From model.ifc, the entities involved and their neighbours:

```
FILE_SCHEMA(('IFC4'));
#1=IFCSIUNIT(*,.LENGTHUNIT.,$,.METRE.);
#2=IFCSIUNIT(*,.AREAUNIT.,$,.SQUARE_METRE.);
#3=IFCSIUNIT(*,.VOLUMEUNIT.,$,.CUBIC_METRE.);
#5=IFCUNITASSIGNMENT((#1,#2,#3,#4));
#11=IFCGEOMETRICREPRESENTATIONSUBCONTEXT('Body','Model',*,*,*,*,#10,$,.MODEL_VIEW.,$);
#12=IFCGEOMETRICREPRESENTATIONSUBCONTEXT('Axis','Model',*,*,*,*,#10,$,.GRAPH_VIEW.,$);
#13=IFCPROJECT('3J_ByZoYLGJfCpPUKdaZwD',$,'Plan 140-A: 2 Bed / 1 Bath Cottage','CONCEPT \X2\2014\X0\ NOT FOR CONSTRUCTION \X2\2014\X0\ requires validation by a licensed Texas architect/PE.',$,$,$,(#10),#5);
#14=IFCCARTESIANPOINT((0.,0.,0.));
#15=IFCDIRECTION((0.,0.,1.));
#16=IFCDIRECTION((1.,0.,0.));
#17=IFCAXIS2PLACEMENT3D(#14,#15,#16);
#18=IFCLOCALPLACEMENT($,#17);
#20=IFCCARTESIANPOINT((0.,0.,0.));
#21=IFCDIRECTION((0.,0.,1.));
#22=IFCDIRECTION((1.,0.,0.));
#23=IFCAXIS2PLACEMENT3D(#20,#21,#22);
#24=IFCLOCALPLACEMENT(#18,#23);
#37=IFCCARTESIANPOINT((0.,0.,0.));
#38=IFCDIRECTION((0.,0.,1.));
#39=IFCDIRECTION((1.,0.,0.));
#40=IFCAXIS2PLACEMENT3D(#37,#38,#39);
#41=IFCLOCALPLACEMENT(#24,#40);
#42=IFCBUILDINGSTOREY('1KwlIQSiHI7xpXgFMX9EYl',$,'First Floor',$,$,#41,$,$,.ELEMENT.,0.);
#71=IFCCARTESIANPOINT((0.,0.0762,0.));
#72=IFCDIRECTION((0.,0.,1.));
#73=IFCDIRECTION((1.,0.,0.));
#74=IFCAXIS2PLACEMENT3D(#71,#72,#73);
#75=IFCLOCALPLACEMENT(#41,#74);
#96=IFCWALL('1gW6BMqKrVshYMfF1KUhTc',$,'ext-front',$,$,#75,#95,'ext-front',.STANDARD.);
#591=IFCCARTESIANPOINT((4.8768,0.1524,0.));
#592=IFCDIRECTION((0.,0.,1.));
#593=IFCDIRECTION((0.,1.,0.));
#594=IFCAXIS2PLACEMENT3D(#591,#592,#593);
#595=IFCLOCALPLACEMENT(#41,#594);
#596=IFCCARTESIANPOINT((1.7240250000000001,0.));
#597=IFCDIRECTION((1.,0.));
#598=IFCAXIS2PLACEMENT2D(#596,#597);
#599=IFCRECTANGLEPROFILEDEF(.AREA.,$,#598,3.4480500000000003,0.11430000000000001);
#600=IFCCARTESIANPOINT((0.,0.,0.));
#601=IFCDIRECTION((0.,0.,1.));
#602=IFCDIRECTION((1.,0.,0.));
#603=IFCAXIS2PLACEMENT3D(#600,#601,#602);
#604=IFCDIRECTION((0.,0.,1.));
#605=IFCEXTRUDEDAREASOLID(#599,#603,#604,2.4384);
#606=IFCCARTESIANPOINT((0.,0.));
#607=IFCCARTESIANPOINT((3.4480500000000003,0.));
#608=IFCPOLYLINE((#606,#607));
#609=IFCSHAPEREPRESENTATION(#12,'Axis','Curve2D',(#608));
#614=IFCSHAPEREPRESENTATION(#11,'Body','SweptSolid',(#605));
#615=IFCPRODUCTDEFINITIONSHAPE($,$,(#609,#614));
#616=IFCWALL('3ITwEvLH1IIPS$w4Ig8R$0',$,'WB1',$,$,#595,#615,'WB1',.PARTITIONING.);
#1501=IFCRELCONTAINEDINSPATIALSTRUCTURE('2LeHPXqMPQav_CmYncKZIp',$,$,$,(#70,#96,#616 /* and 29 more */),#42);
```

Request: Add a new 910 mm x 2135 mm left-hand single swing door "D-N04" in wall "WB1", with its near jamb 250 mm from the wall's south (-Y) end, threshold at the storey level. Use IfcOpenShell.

```python
import numpy as np
import ifcopenshell
import ifcopenshell.api.feature
import ifcopenshell.api.geometry
import ifcopenshell.api.root
import ifcopenshell.api.spatial
import ifcopenshell.geom
import ifcopenshell.util.element
import ifcopenshell.util.placement
import ifcopenshell.util.representation
import ifcopenshell.util.shape
import ifcopenshell.util.unit

model = ifcopenshell.open("model.ifc")
unit_scale = ifcopenshell.util.unit.calculate_unit_scale(model)
settings = ifcopenshell.geom.settings()


def volume(element):
    """Net volume in cubic metres, openings subtracted."""
    shape = ifcopenshell.geom.create_shape(settings, element)
    return ifcopenshell.util.shape.get_volume(shape.geometry)


wall = model.by_id(616)
storey = ifcopenshell.util.element.get_container(wall, ifc_class="IfcBuildingStorey")
context = ifcopenshell.util.representation.get_context(model, "Model", "Body", "MODEL_VIEW")
before = volume(wall)

width, height, from_end, sill = 0.91, 2.135, 0.25, 0.0  # metres

# The wall runs along its own X axis, and the end named is its -X end.
wall_shape = ifcopenshell.geom.create_shape(settings, wall)
x, y, z = ifcopenshell.util.shape.get_vertices(wall_shape.geometry).T
start = x.min() + from_end
face, thickness = float(y.min()), float(y.max() - y.min())
wall_matrix = ifcopenshell.util.placement.get_local_placement(wall.ObjectPlacement)
level = ifcopenshell.util.placement.get_local_placement(storey.ObjectPlacement)[2, 3]


def in_wall(x, y):
    """Placement at x, y metres in the wall's axes, at sill height."""
    matrix = wall_matrix.copy()
    matrix[:, 3] = wall_matrix @ np.array([x / unit_scale, y / unit_scale, 0.0, 1.0])
    matrix[2, 3] = level + sill / unit_scale
    return matrix


# Opening: a box that overshoots both wall faces by 50 mm.
opening = ifcopenshell.api.root.create_entity(model, ifc_class="IfcOpeningElement", predefined_type="OPENING")
box = ifcopenshell.api.geometry.add_wall_representation(
    model, context=context, length=width, height=height, thickness=thickness + 0.1
)
ifcopenshell.api.geometry.assign_representation(model, product=opening, representation=box)
ifcopenshell.api.geometry.edit_object_placement(model, product=opening, matrix=in_wall(start, face - 0.05), is_si=False)
ifcopenshell.api.feature.add_feature(model, feature=opening, element=wall)

door = ifcopenshell.api.root.create_entity(model, ifc_class="IfcDoor", name="D-N04", predefined_type="DOOR")
door.OverallWidth, door.OverallHeight = width / unit_scale, height / unit_scale
door.OperationType = "SINGLE_SWING_LEFT"
body = ifcopenshell.api.geometry.add_door_representation(
    model,
    context=context,
    overall_width=door.OverallWidth,
    overall_height=door.OverallHeight,
    operation_type="SINGLE_SWING_LEFT",
    lining_properties={"LiningDepth": thickness / unit_scale, "ThresholdDepth": thickness / unit_scale},
)
ifcopenshell.api.geometry.assign_representation(model, product=door, representation=body)
ifcopenshell.api.spatial.assign_container(model, products=[door], relating_structure=storey)
ifcopenshell.api.feature.add_filling(model, opening=opening, element=door)

# The lining spans the wall, so the door starts at the wall face.
ifcopenshell.api.geometry.edit_object_placement(model, product=door, matrix=in_wall(start, face), is_si=False)

after = volume(wall)

print(f"wall volume {before:.3f} -> {after:.3f} m3")

model.write("model_rev.ifc")
```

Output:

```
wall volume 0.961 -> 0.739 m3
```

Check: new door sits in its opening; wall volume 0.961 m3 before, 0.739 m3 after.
